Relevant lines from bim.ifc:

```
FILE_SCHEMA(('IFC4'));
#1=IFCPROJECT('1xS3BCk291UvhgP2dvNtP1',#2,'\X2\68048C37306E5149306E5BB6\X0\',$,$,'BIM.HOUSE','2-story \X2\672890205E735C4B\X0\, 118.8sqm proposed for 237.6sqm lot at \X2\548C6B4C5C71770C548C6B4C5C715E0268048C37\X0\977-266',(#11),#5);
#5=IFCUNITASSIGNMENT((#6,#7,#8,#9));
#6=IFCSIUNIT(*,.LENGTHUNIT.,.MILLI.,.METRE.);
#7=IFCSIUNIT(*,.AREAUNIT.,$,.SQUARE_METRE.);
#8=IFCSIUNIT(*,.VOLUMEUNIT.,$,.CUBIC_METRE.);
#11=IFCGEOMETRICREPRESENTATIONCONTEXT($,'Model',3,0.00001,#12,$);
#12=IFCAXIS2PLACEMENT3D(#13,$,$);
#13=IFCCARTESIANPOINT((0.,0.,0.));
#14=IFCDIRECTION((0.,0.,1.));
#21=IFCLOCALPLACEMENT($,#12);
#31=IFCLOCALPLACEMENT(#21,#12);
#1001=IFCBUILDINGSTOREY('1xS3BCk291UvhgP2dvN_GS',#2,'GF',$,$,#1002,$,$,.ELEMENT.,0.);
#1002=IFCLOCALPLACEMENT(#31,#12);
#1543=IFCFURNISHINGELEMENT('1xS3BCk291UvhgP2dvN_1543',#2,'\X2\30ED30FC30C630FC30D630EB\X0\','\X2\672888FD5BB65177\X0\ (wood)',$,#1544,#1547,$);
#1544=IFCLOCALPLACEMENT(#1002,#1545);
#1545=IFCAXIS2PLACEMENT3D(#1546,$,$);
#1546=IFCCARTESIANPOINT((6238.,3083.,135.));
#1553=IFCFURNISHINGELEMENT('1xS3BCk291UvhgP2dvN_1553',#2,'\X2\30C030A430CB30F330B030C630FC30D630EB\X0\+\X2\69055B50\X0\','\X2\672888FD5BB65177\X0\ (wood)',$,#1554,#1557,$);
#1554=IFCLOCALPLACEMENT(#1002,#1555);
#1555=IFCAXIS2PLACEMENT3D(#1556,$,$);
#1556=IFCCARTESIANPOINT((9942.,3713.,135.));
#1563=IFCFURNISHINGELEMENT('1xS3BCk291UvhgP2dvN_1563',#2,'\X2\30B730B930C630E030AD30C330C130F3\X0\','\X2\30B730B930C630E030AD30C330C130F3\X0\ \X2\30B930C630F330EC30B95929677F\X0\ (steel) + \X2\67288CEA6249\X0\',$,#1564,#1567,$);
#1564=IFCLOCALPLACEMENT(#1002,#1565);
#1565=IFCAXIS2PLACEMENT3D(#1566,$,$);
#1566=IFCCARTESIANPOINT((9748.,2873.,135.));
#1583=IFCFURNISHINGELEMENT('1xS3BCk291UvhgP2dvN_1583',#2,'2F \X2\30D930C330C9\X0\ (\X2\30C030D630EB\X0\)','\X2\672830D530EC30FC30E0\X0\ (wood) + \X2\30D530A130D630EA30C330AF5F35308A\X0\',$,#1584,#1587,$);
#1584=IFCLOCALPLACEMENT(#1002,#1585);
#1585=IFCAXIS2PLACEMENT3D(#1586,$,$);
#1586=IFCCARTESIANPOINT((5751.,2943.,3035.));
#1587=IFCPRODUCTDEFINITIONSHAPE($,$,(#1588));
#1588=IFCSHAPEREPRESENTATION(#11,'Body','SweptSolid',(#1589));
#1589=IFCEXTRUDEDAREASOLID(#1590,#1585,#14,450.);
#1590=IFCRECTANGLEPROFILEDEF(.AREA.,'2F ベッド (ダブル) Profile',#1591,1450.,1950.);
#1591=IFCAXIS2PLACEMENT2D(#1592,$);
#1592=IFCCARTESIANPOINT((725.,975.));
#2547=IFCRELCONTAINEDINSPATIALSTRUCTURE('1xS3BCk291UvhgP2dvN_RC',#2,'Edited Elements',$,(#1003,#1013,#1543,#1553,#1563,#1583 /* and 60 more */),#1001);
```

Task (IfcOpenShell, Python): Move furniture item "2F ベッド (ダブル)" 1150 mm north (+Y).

```python
import ifcopenshell
import ifcopenshell.api.geometry
import ifcopenshell.util.placement

model = ifcopenshell.open("bim.ifc")

item = model.by_guid("1xS3BCk291UvhgP2dvN_1583")
matrix = ifcopenshell.util.placement.get_local_placement(item.ObjectPlacement)
matrix[1, 3] += 1150.0
ifcopenshell.api.geometry.edit_object_placement(model, product=item, matrix=matrix, is_si=False)

print(ifcopenshell.util.placement.get_local_placement(item.ObjectPlacement).round(3) + 0.0)

model.write("bim_rev.ifc")
```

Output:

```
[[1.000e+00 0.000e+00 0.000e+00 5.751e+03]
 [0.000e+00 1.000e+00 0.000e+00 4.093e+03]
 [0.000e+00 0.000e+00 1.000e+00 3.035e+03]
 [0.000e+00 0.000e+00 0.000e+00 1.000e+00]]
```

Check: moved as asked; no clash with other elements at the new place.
